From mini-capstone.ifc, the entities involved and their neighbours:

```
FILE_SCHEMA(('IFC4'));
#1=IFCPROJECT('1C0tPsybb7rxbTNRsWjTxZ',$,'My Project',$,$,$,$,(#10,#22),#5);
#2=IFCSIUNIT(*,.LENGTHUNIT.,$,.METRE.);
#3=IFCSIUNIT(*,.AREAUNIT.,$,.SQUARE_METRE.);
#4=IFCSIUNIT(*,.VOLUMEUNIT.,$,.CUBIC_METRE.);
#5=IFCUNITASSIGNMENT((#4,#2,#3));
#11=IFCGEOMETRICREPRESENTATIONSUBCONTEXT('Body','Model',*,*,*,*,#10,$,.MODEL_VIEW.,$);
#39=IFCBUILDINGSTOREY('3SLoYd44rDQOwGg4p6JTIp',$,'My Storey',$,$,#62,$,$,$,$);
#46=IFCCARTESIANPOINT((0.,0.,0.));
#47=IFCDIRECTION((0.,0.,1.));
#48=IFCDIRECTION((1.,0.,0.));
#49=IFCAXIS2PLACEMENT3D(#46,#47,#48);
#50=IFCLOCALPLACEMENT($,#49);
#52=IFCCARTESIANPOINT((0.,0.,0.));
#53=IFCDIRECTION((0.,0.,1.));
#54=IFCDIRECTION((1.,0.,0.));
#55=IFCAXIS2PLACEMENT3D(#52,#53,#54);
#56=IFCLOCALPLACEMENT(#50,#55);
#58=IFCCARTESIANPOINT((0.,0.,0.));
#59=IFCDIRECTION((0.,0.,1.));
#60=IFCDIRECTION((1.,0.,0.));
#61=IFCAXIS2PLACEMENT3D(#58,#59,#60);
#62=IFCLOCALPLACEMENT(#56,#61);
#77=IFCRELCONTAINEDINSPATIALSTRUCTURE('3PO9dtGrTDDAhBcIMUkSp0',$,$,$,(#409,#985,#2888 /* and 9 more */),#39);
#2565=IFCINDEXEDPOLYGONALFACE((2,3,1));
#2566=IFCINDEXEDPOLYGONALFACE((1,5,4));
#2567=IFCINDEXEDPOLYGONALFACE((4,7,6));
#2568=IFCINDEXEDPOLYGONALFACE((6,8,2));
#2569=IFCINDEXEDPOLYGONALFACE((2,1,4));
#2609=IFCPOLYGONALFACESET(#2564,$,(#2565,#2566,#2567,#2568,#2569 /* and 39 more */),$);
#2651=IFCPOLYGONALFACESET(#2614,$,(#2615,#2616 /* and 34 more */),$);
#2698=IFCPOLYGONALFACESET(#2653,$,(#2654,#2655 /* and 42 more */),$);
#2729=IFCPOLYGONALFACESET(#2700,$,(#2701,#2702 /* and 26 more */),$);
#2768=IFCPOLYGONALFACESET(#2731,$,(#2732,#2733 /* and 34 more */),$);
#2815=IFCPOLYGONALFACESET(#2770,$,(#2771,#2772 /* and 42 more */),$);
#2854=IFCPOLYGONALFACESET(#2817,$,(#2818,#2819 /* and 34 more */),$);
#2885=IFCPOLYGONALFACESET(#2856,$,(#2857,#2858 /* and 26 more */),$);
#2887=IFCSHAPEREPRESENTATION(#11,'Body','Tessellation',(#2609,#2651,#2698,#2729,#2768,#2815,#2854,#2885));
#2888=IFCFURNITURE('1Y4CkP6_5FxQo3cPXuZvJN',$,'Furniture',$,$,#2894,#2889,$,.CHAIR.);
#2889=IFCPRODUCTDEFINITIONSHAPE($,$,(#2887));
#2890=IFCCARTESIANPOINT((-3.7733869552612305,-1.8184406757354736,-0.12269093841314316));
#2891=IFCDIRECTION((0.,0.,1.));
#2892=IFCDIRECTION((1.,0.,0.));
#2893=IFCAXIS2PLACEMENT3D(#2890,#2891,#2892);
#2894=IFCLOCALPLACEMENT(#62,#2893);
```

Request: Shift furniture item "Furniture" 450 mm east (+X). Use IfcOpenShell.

```python
import ifcopenshell
import ifcopenshell.api.geometry
import ifcopenshell.util.placement
import ifcopenshell.util.unit

model = ifcopenshell.open("mini-capstone.ifc")
unit_scale = ifcopenshell.util.unit.calculate_unit_scale(model)

item = model.by_guid("1Y4CkP6_5FxQo3cPXuZvJN")
matrix = ifcopenshell.util.placement.get_local_placement(item.ObjectPlacement)
matrix[0, 3] += 0.45 / unit_scale
ifcopenshell.api.geometry.edit_object_placement(model, product=item, matrix=matrix, is_si=False)

print(ifcopenshell.util.placement.get_local_placement(item.ObjectPlacement).round(3) + 0.0)

model.write("mini-capstone_v2.ifc")
```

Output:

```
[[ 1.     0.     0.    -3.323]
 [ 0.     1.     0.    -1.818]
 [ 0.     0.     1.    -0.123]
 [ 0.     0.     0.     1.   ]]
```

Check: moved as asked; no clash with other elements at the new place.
